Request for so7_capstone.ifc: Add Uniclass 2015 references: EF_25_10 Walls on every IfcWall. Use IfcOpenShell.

First a look at what the model holds.

```python
import ifcopenshell

model = ifcopenshell.open("so7_capstone.ifc")
print(model.schema)
print("classifications:", [c.Name for c in model.by_type("IfcClassification")])
for ifc_class in ("IfcDoor", "IfcRoof", "IfcStair", "IfcWall", "IfcWindow"):
    print(ifc_class, len(model.by_type(ifc_class)))
```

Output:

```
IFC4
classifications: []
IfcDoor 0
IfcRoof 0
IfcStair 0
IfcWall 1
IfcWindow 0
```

```python
import ifcopenshell
import ifcopenshell.api.classification

model = ifcopenshell.open("so7_capstone.ifc")

system = ifcopenshell.api.classification.add_classification(model, classification="Uniclass 2015")

codes = {
    "IfcWall": ("EF_25_10", "Walls"),
}
for ifc_class, (code, name) in codes.items():
    products = model.by_type(ifc_class)
    ifcopenshell.api.classification.add_reference(
        model, products=products, classification=system, identification=code, name=name
    )
    print(code, len(products))

model.write("so7_capstone_rev.ifc")
```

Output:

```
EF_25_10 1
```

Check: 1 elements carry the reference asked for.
